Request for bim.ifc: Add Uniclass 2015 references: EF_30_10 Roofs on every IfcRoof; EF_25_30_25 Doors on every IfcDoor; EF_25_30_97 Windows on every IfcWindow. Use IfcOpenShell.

First a look at what the model holds.

```python
import ifcopenshell

model = ifcopenshell.open("bim.ifc")
print(model.schema)
print("classifications:", [c.Name for c in model.by_type("IfcClassification")])
for ifc_class in ("IfcDoor", "IfcRoof", "IfcStair", "IfcWall", "IfcWindow"):
    print(ifc_class, len(model.by_type(ifc_class)))
```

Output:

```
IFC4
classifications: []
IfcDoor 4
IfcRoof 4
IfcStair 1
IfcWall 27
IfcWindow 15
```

```python
import ifcopenshell
import ifcopenshell.api.classification

model = ifcopenshell.open("bim.ifc")

system = ifcopenshell.api.classification.add_classification(model, classification="Uniclass 2015")

codes = {
    "IfcRoof": ("EF_30_10", "Roofs"),
    "IfcDoor": ("EF_25_30_25", "Doors"),
    "IfcWindow": ("EF_25_30_97", "Windows"),
}
for ifc_class, (code, name) in codes.items():
    products = model.by_type(ifc_class)
    ifcopenshell.api.classification.add_reference(
        model, products=products, classification=system, identification=code, name=name
    )
    print(code, len(products))

model.write("bim_rev.ifc")
```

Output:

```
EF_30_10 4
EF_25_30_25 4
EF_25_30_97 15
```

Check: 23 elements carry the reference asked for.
